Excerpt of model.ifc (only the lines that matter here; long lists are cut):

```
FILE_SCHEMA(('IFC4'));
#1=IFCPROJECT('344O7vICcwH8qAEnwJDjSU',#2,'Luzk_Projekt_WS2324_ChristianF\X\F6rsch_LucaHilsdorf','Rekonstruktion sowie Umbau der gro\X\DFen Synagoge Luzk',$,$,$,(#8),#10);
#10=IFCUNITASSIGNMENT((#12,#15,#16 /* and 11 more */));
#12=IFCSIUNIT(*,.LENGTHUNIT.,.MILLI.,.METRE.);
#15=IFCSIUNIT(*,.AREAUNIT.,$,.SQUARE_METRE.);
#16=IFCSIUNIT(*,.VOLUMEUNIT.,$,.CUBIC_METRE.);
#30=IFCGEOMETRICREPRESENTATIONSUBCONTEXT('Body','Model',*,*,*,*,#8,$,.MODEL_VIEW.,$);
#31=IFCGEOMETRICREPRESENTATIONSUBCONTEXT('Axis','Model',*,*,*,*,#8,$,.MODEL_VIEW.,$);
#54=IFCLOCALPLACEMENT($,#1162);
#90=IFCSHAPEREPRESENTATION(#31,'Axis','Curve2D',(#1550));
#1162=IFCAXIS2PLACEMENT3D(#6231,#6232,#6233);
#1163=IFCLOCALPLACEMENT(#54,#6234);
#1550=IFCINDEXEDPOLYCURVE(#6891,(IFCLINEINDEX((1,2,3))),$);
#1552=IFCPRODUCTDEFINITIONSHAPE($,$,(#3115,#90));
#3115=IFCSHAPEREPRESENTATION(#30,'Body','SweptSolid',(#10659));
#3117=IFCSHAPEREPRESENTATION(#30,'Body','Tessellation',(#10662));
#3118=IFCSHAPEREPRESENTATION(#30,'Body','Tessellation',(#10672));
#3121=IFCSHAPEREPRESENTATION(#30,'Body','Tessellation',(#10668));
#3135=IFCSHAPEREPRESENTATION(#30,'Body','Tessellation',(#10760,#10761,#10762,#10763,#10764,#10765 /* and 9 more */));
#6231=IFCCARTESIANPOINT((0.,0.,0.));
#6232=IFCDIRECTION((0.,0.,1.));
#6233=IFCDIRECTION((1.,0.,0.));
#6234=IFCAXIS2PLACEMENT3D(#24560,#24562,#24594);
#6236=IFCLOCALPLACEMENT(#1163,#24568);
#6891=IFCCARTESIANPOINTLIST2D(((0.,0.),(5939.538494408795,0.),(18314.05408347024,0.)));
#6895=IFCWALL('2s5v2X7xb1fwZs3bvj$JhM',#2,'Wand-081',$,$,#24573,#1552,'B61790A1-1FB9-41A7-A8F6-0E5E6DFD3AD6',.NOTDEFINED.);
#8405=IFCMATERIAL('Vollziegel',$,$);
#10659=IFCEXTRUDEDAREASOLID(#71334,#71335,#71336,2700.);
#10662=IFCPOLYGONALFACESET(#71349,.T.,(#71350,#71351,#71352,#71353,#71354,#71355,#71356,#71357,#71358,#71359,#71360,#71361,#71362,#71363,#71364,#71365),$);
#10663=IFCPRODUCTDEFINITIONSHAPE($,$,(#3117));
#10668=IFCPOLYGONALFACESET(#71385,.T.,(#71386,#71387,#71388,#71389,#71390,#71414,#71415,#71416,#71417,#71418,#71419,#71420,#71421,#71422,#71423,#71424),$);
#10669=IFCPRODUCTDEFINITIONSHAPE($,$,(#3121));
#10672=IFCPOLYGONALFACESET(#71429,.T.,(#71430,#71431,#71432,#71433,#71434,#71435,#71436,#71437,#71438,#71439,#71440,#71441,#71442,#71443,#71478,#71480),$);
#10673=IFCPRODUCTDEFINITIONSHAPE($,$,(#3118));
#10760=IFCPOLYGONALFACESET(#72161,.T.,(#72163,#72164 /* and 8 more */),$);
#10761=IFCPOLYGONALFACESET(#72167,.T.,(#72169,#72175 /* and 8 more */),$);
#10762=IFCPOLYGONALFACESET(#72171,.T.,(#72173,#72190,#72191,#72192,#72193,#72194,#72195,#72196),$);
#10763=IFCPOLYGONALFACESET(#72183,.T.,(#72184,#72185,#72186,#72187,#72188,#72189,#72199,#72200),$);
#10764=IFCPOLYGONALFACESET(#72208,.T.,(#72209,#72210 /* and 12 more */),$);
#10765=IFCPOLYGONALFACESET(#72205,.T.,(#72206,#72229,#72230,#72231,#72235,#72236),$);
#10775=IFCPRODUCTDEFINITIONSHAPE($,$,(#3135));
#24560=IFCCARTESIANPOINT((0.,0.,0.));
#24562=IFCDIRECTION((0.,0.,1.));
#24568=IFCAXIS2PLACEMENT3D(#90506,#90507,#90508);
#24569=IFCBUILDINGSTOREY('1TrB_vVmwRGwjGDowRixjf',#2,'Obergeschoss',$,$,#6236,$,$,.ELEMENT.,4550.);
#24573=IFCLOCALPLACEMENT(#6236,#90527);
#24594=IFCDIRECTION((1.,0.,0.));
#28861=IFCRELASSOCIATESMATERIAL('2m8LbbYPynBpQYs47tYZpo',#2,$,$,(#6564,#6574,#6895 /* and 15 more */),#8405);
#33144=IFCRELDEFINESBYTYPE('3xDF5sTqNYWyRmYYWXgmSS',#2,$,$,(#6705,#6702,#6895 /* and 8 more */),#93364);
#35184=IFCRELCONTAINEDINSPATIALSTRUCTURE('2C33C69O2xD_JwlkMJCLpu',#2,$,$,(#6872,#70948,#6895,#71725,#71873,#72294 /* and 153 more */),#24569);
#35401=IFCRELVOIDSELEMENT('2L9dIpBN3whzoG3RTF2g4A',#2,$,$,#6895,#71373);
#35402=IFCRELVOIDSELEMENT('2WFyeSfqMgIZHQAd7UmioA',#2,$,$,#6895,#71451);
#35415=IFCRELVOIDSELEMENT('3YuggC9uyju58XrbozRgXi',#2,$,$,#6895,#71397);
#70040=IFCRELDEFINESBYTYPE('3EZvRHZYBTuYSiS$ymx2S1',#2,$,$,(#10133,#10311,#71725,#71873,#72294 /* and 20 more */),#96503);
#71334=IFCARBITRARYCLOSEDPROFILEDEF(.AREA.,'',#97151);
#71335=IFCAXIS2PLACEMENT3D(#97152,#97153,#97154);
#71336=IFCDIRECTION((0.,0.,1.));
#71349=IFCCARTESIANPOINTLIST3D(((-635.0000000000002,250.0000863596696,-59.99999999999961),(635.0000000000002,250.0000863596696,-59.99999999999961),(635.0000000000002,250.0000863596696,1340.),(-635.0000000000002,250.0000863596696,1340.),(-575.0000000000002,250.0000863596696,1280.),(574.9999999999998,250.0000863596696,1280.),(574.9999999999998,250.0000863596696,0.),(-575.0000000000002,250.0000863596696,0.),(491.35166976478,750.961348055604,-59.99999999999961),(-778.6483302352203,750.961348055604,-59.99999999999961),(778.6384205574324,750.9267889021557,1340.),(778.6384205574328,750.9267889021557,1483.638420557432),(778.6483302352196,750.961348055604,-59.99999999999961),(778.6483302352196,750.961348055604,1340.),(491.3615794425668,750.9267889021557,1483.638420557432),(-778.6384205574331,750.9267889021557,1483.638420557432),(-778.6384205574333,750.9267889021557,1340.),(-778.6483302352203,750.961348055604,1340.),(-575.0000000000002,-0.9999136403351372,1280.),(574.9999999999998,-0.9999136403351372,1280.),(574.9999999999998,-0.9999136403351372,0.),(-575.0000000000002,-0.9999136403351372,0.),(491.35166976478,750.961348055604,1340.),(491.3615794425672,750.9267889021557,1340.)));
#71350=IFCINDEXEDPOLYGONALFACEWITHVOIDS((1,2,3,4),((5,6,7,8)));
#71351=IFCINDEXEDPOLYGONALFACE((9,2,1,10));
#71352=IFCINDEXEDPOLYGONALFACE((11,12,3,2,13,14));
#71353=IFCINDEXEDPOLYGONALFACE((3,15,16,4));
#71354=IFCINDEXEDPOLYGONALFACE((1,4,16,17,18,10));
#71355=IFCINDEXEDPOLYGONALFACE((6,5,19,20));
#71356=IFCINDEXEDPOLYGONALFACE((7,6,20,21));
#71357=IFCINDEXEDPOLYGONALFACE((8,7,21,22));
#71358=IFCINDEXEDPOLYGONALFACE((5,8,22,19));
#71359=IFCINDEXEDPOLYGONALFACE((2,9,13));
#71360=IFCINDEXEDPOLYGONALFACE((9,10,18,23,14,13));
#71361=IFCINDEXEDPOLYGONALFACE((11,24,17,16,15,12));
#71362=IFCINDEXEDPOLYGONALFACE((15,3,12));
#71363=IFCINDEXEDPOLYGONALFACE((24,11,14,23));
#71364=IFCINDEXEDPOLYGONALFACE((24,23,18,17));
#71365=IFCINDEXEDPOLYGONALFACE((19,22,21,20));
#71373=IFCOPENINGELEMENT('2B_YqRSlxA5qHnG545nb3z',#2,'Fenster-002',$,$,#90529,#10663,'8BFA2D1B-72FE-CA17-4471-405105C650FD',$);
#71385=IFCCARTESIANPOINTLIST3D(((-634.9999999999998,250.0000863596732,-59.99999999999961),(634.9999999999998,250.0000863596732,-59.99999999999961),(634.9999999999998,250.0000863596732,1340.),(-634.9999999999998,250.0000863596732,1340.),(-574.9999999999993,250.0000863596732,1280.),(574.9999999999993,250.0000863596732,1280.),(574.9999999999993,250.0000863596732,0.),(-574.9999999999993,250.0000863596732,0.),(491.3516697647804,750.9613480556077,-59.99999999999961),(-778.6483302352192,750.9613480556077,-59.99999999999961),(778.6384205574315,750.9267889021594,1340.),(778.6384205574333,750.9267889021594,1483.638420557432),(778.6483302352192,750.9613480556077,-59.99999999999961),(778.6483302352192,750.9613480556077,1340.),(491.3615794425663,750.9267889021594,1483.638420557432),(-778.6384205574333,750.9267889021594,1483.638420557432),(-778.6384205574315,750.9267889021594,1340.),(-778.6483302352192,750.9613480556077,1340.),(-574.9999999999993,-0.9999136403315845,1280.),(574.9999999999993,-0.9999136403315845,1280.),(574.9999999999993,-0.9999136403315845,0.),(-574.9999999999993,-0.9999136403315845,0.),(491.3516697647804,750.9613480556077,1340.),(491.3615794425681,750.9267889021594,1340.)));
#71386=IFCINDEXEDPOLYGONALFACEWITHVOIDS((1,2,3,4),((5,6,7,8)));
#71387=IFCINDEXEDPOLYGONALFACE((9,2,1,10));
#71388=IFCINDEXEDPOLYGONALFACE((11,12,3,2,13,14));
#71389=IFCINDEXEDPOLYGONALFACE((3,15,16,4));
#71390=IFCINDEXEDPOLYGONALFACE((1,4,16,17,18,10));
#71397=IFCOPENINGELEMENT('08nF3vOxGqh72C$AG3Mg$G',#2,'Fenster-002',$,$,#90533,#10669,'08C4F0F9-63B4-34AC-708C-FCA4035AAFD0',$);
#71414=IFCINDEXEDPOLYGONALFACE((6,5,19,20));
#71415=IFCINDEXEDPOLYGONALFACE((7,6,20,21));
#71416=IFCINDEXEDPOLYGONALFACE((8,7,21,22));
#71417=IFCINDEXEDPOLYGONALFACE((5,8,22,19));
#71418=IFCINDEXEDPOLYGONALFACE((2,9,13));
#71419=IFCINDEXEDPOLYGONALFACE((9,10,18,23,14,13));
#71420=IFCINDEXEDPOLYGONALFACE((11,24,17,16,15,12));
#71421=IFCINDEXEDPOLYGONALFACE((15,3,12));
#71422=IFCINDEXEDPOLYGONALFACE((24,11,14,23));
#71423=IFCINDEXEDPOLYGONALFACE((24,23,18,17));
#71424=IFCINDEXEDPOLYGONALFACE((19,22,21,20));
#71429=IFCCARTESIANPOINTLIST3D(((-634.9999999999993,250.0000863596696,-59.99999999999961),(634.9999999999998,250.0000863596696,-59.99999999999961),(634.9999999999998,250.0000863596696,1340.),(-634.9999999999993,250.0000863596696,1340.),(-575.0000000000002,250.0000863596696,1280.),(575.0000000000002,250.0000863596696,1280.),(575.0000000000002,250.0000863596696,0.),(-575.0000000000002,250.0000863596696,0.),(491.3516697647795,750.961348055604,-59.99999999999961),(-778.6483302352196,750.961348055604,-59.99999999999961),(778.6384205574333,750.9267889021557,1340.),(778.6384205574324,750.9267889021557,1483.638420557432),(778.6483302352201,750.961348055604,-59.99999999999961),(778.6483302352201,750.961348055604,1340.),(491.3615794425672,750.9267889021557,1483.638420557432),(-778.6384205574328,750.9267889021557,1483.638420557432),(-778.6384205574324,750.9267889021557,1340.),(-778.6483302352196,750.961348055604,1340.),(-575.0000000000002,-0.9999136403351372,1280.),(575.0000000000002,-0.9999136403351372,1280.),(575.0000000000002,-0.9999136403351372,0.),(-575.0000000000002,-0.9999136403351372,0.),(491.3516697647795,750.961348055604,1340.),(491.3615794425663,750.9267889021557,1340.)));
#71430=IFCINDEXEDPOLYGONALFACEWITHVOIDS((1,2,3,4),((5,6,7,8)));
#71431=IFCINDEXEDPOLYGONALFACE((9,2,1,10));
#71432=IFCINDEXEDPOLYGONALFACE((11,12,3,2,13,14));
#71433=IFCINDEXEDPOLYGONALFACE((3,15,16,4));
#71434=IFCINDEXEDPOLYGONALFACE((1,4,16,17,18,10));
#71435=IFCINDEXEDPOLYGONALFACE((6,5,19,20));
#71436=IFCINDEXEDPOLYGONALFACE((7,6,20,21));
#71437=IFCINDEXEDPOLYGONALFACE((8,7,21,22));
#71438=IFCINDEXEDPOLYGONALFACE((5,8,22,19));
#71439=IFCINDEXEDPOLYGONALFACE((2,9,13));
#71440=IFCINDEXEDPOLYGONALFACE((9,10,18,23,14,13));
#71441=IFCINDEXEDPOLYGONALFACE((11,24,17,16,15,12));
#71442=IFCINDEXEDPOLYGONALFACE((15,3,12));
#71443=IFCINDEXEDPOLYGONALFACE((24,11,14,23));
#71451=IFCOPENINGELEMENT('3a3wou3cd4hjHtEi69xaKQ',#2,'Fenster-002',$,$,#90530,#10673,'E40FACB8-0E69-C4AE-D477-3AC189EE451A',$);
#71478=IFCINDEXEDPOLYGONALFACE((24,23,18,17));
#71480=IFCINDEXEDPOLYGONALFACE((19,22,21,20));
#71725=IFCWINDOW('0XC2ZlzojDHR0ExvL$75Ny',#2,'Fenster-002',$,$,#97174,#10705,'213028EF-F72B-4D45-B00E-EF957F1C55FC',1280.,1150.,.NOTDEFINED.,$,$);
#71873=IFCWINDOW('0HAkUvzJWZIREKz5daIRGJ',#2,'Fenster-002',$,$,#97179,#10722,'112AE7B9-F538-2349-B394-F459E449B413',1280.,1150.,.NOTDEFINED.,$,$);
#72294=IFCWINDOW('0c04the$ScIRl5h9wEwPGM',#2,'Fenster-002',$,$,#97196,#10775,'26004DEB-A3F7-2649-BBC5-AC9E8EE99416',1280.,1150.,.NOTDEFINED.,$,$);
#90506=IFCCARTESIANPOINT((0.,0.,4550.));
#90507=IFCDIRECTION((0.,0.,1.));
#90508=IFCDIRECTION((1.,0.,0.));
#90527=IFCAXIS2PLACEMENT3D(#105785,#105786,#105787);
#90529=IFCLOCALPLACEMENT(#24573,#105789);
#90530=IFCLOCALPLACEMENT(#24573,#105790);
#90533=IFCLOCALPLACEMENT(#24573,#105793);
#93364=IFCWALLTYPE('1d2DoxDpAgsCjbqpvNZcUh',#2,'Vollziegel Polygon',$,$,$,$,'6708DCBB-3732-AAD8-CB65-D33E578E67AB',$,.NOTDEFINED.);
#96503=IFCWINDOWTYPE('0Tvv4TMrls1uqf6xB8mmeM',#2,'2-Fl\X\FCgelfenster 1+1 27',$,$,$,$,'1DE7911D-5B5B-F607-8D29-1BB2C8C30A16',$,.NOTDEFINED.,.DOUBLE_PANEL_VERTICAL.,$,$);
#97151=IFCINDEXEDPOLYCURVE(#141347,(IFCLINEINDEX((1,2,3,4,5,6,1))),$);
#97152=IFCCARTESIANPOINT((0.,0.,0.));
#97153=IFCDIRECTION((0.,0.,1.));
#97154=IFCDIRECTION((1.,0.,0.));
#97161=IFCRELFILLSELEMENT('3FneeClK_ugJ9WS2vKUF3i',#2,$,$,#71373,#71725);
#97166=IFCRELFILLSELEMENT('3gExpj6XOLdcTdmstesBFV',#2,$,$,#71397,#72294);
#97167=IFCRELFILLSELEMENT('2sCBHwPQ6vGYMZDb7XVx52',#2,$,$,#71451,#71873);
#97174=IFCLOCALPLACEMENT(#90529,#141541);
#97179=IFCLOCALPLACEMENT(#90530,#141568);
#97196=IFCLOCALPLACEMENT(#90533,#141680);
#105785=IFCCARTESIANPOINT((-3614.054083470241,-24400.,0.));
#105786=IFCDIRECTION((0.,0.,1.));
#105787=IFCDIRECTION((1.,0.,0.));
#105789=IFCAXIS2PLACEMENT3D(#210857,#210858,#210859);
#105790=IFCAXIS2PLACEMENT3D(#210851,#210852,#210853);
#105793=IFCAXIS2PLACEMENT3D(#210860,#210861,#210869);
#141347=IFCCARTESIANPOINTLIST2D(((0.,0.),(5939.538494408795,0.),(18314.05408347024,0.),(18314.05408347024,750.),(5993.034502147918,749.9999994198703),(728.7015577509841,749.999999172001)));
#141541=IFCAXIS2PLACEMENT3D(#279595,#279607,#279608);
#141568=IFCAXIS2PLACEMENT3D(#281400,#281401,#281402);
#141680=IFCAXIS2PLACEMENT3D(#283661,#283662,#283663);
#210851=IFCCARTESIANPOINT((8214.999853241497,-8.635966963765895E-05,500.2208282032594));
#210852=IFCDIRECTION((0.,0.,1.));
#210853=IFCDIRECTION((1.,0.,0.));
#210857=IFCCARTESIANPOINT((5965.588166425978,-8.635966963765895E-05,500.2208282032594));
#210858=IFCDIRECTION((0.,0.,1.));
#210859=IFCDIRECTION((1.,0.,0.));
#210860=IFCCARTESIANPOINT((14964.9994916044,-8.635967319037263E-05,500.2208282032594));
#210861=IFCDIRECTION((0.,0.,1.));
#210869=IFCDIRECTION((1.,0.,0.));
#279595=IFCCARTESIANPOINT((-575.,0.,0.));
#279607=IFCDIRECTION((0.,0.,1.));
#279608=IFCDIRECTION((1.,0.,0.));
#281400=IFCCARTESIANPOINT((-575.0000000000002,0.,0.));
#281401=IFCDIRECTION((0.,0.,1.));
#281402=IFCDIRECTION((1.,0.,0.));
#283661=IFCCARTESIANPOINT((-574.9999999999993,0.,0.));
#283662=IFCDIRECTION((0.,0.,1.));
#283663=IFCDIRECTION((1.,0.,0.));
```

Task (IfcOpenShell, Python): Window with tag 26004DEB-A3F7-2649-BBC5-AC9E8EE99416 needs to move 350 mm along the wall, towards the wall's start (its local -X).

```python
import ifcopenshell
import ifcopenshell.api.geometry
import ifcopenshell.util.placement
import ifcopenshell.util.unit

model = ifcopenshell.open("model.ifc")
unit_scale = ifcopenshell.util.unit.calculate_unit_scale(model)

window = model.by_guid("0c04the$ScIRl5h9wEwPGM")
opening = window.FillsVoids[0].RelatingOpeningElement
wall = opening.VoidsElements[0].RelatingBuildingElement

wall_matrix = ifcopenshell.util.placement.get_local_placement(wall.ObjectPlacement)
shift = wall_matrix[:3, 0] * -0.35 / unit_scale
before = ifcopenshell.util.placement.get_local_placement(window.ObjectPlacement)[:3, 3].copy()

# The window is placed relative to its opening, so it follows when the opening moves.
matrix = ifcopenshell.util.placement.get_local_placement(opening.ObjectPlacement)
matrix[:3, 3] += shift
ifcopenshell.api.geometry.edit_object_placement(
    model, product=opening, matrix=matrix, is_si=False, should_transform_children=True
)

after = ifcopenshell.util.placement.get_local_placement(window.ObjectPlacement)[:3, 3]
print("window moved by", (after - before).round(3) + 0.0)

model.write("model_rev.ifc")
```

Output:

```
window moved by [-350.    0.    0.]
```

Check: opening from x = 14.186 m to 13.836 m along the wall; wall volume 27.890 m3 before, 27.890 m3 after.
